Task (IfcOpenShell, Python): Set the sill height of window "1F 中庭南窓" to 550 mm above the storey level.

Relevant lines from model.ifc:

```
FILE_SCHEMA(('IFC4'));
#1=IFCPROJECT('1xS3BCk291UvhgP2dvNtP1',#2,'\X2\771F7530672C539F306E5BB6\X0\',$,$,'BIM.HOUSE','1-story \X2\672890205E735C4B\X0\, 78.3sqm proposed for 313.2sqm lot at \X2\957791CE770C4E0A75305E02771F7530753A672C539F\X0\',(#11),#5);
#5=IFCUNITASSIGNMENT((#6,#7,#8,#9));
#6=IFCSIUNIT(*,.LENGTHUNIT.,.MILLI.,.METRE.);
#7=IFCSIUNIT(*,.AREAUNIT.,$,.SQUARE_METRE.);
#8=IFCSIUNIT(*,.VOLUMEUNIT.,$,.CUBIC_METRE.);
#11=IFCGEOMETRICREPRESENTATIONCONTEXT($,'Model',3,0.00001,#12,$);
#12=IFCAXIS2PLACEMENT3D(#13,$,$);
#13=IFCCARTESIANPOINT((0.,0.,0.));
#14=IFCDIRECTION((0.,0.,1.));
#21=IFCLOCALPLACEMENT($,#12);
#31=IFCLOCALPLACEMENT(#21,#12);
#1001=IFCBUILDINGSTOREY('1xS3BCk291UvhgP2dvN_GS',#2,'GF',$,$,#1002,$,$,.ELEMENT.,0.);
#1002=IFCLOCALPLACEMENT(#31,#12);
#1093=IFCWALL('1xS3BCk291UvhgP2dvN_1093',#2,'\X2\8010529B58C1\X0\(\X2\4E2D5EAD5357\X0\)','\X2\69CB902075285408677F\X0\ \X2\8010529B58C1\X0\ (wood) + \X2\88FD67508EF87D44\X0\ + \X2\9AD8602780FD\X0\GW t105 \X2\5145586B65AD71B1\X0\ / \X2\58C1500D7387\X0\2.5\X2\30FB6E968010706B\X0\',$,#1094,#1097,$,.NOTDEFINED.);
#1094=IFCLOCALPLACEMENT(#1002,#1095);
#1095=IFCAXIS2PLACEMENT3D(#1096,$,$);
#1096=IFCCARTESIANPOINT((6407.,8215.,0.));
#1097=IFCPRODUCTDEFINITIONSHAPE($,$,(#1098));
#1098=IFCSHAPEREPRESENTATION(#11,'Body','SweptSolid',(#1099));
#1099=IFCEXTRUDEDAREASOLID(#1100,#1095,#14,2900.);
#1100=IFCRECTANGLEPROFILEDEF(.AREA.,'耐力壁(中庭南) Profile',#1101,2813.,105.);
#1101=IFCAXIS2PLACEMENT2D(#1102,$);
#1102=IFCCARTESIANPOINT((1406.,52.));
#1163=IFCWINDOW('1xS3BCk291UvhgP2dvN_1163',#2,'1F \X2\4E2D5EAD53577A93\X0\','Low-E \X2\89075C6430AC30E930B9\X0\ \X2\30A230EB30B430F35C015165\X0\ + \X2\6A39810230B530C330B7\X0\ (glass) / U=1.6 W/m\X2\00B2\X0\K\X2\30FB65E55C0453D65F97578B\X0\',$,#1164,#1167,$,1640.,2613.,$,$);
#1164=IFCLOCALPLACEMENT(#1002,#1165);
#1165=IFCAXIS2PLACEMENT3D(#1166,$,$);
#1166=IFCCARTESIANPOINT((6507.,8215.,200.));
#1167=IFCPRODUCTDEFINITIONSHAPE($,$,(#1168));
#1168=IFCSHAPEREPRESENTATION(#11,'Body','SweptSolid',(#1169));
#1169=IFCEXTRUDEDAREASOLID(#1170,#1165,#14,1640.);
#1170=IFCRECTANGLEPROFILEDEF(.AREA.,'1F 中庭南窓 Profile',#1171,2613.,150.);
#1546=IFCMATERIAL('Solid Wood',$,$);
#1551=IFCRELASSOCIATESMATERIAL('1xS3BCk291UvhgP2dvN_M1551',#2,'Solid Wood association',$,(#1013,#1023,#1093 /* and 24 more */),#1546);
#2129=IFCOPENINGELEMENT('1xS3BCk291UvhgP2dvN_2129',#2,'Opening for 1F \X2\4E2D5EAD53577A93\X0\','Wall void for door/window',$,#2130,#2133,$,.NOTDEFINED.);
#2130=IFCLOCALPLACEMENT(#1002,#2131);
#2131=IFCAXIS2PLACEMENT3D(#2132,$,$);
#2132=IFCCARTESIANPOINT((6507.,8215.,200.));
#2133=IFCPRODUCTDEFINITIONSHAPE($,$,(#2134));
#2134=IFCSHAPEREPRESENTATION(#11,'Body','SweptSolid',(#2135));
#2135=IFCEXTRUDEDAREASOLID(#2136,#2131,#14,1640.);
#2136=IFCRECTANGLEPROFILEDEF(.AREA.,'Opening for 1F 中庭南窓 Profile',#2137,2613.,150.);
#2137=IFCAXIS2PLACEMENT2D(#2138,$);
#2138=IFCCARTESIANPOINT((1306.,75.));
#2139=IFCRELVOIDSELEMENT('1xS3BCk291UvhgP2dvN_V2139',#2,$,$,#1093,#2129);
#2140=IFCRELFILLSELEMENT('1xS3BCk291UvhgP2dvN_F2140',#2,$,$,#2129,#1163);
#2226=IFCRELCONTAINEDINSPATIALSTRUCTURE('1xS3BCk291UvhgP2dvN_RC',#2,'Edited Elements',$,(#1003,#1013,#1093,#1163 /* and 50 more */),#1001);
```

```python
import numpy as np
import ifcopenshell
import ifcopenshell.api.geometry
import ifcopenshell.geom
import ifcopenshell.util.element
import ifcopenshell.util.placement
import ifcopenshell.util.shape
import ifcopenshell.util.unit

model = ifcopenshell.open("model.ifc")
unit_scale = ifcopenshell.util.unit.calculate_unit_scale(model)

window = model.by_guid("1xS3BCk291UvhgP2dvN_1163")
opening = window.FillsVoids[0].RelatingOpeningElement
storey = ifcopenshell.util.element.get_container(window, ifc_class="IfcBuildingStorey")
level = ifcopenshell.util.placement.get_local_placement(storey.ObjectPlacement)[2, 3]

# The opening's origin need not be at the sill, so measure its lowest point.
shape = ifcopenshell.geom.create_shape(ifcopenshell.geom.settings(), opening)
bottom = ifcopenshell.util.shape.get_shape_bottom_elevation(shape, shape.geometry) / unit_scale
dz = level + 550.0 - bottom

shift = np.array([0.0, 0.0, dz])
# The window is not placed relative to its opening, so move both.
for product in (opening, window):
    matrix = ifcopenshell.util.placement.get_local_placement(product.ObjectPlacement)
    matrix[:3, 3] += shift
    ifcopenshell.api.geometry.edit_object_placement(model, product=product, matrix=matrix, is_si=False)

print(f"moved by {dz * unit_scale:+.3f} m")

model.write("model_rev.ifc")
```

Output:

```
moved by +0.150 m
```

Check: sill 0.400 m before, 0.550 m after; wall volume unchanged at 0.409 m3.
